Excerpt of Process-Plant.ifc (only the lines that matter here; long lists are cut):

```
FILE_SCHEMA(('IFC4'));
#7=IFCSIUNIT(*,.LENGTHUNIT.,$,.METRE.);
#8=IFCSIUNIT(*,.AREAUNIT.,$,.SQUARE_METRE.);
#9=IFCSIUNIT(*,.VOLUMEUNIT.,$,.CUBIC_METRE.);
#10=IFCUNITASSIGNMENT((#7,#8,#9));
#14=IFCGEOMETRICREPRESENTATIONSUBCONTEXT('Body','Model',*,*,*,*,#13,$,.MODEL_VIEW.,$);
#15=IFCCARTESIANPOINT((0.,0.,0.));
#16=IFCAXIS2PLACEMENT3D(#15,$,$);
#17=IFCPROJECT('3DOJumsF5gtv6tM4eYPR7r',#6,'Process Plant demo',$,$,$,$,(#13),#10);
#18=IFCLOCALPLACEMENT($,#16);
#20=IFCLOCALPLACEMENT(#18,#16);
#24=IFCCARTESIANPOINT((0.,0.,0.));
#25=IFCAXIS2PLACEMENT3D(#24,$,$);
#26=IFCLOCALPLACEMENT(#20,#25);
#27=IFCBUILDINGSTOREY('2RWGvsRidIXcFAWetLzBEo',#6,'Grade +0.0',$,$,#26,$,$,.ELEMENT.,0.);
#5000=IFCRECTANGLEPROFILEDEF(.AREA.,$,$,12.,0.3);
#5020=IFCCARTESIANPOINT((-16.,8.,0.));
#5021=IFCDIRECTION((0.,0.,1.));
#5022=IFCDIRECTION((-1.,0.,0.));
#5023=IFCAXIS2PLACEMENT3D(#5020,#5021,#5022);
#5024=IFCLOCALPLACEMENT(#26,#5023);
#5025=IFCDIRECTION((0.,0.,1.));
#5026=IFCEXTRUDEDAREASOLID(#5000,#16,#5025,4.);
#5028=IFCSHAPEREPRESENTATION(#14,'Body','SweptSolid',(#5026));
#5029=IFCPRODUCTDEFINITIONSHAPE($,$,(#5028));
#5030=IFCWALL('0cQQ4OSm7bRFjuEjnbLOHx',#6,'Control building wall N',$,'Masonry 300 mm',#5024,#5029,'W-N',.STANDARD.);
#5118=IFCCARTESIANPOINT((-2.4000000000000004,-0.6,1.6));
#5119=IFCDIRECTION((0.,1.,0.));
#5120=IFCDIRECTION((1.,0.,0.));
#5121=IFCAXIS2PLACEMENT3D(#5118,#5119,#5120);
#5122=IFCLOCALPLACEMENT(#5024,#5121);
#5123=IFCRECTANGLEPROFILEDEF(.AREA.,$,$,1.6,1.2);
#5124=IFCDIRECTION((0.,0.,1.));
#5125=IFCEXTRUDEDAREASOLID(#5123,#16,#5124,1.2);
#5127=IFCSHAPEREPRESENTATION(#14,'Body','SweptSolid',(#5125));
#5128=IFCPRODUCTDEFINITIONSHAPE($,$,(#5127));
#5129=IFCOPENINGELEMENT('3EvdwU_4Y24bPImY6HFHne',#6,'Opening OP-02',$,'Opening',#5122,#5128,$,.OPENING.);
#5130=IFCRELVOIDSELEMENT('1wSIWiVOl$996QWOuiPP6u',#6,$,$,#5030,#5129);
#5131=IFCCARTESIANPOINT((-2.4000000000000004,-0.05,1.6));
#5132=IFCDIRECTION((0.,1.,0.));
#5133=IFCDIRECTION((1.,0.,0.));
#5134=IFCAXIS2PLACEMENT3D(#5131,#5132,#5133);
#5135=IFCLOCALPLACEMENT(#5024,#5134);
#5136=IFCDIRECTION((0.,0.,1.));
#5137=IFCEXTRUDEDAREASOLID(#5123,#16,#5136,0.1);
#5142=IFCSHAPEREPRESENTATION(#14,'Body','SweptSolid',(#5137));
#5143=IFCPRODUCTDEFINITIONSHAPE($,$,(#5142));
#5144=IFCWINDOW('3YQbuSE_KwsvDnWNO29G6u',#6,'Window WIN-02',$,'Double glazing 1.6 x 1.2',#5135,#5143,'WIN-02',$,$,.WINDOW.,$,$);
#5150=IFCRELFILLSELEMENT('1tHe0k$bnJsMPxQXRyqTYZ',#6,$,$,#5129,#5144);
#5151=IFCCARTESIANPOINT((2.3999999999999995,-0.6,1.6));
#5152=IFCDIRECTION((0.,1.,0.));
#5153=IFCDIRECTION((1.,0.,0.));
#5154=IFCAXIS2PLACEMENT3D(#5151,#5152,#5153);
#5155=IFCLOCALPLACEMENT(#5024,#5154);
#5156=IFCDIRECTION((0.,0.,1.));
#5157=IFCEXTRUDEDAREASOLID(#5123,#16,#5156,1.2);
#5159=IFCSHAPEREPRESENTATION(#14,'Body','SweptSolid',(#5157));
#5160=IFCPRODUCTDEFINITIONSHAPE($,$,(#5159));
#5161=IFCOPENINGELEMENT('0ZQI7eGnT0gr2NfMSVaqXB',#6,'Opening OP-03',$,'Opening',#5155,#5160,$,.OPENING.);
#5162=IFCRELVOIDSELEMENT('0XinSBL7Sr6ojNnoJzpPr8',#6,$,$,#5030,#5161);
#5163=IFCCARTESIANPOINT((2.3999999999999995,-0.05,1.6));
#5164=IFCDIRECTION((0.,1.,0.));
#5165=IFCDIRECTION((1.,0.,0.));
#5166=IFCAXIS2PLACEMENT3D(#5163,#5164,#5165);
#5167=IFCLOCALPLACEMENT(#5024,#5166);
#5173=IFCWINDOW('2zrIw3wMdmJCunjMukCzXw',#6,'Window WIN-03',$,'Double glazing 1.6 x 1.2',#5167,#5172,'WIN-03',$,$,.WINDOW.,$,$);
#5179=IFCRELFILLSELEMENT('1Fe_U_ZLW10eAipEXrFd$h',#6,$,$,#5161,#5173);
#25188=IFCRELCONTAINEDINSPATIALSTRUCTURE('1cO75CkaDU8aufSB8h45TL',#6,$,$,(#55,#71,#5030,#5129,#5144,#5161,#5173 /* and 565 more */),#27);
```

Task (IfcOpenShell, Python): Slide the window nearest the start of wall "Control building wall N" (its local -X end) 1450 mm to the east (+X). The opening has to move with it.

```python
import ifcopenshell
import ifcopenshell.api.geometry
import ifcopenshell.util.placement

model = ifcopenshell.open("Process-Plant.ifc")

window = model.by_guid("3YQbuSE_KwsvDnWNO29G6u")
opening = window.FillsVoids[0].RelatingOpeningElement
wall = opening.VoidsElements[0].RelatingBuildingElement

wall_matrix = ifcopenshell.util.placement.get_local_placement(wall.ObjectPlacement)
shift = wall_matrix[:3, 0] * -1.45
before = ifcopenshell.util.placement.get_local_placement(window.ObjectPlacement)[:3, 3].copy()

# The window is not placed relative to its opening, so move both.
for product in (opening, window):
    matrix = ifcopenshell.util.placement.get_local_placement(product.ObjectPlacement)
    matrix[:3, 3] += shift
    ifcopenshell.api.geometry.edit_object_placement(model, product=product, matrix=matrix, is_si=False)

after = ifcopenshell.util.placement.get_local_placement(window.ObjectPlacement)[:3, 3]
print("window moved by", (after - before).round(3) + 0.0)

model.write("Process-Plant_v2.ifc")
```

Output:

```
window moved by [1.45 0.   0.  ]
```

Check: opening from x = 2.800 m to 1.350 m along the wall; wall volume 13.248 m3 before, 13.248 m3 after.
